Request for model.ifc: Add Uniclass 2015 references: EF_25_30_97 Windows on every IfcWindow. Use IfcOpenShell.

First a look at what the model holds.

```python
import ifcopenshell

model = ifcopenshell.open("model.ifc")
print(model.schema)
print("classifications:", [c.Name for c in model.by_type("IfcClassification")])
for ifc_class in ("IfcDoor", "IfcRoof", "IfcStair", "IfcWall", "IfcWindow"):
    print(ifc_class, len(model.by_type(ifc_class)))
```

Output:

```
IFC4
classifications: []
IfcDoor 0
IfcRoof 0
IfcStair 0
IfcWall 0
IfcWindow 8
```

```python
import ifcopenshell
import ifcopenshell.api.classification

model = ifcopenshell.open("model.ifc")

system = ifcopenshell.api.classification.add_classification(model, classification="Uniclass 2015")

codes = {
    "IfcWindow": ("EF_25_30_97", "Windows"),
}
for ifc_class, (code, name) in codes.items():
    products = model.by_type(ifc_class)
    ifcopenshell.api.classification.add_reference(
        model, products=products, classification=system, identification=code, name=name
    )
    print(code, len(products))

model.write("model_v2.ifc")
```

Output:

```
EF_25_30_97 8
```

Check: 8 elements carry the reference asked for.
